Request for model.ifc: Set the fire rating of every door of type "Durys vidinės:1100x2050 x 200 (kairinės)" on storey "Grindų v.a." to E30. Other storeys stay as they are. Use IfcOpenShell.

First a look at what the model holds.

```python
import ifcopenshell
import ifcopenshell.util.element

model = ifcopenshell.open("model.ifc")
print(model.schema)
storey = next(s for s in model.by_type("IfcBuildingStorey") if s.Name == "Grindų v.a.")
doors = [e for e in ifcopenshell.util.element.get_decomposition(storey) if e.is_a("IfcDoor")]
seen = {}
for e in doors:
    element_type = ifcopenshell.util.element.get_type(e)
    key = (element_type.Name if element_type != e and element_type else None, ifcopenshell.util.element.get_pset(e, "Pset_DoorCommon", "FireRating"))
    seen[key] = seen.get(key, 0) + 1
for (name, value), count in sorted(seen.items(), key=str):
    print(count, "x", name, "|", value)
```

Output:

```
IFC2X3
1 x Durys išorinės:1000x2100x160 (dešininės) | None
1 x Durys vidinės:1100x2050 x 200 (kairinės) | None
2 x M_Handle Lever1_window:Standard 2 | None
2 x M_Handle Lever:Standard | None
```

```python
import ifcopenshell
import ifcopenshell.api.pset
import ifcopenshell.util.element

model = ifcopenshell.open("model.ifc")

storey = next(s for s in model.by_type("IfcBuildingStorey") if s.Name == "Grindų v.a.")
doors = [e for e in ifcopenshell.util.element.get_decomposition(storey) if e.is_a("IfcDoor")]

count = 0
for e in doors:
    element_type = ifcopenshell.util.element.get_type(e)
    if element_type in (None, e) or element_type.Name != "Durys vidinės:1100x2050 x 200 (kairinės)":
        continue
    # add_pset returns the element's existing set when there is one.
    pset = ifcopenshell.api.pset.add_pset(model, product=e, name="Pset_DoorCommon")
    ifcopenshell.api.pset.edit_pset(model, pset=pset, properties={"FireRating": "E30"})
    count += 1

print(count, "doors updated")

model.write("model_rev.ifc")
```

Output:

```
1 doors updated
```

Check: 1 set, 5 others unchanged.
